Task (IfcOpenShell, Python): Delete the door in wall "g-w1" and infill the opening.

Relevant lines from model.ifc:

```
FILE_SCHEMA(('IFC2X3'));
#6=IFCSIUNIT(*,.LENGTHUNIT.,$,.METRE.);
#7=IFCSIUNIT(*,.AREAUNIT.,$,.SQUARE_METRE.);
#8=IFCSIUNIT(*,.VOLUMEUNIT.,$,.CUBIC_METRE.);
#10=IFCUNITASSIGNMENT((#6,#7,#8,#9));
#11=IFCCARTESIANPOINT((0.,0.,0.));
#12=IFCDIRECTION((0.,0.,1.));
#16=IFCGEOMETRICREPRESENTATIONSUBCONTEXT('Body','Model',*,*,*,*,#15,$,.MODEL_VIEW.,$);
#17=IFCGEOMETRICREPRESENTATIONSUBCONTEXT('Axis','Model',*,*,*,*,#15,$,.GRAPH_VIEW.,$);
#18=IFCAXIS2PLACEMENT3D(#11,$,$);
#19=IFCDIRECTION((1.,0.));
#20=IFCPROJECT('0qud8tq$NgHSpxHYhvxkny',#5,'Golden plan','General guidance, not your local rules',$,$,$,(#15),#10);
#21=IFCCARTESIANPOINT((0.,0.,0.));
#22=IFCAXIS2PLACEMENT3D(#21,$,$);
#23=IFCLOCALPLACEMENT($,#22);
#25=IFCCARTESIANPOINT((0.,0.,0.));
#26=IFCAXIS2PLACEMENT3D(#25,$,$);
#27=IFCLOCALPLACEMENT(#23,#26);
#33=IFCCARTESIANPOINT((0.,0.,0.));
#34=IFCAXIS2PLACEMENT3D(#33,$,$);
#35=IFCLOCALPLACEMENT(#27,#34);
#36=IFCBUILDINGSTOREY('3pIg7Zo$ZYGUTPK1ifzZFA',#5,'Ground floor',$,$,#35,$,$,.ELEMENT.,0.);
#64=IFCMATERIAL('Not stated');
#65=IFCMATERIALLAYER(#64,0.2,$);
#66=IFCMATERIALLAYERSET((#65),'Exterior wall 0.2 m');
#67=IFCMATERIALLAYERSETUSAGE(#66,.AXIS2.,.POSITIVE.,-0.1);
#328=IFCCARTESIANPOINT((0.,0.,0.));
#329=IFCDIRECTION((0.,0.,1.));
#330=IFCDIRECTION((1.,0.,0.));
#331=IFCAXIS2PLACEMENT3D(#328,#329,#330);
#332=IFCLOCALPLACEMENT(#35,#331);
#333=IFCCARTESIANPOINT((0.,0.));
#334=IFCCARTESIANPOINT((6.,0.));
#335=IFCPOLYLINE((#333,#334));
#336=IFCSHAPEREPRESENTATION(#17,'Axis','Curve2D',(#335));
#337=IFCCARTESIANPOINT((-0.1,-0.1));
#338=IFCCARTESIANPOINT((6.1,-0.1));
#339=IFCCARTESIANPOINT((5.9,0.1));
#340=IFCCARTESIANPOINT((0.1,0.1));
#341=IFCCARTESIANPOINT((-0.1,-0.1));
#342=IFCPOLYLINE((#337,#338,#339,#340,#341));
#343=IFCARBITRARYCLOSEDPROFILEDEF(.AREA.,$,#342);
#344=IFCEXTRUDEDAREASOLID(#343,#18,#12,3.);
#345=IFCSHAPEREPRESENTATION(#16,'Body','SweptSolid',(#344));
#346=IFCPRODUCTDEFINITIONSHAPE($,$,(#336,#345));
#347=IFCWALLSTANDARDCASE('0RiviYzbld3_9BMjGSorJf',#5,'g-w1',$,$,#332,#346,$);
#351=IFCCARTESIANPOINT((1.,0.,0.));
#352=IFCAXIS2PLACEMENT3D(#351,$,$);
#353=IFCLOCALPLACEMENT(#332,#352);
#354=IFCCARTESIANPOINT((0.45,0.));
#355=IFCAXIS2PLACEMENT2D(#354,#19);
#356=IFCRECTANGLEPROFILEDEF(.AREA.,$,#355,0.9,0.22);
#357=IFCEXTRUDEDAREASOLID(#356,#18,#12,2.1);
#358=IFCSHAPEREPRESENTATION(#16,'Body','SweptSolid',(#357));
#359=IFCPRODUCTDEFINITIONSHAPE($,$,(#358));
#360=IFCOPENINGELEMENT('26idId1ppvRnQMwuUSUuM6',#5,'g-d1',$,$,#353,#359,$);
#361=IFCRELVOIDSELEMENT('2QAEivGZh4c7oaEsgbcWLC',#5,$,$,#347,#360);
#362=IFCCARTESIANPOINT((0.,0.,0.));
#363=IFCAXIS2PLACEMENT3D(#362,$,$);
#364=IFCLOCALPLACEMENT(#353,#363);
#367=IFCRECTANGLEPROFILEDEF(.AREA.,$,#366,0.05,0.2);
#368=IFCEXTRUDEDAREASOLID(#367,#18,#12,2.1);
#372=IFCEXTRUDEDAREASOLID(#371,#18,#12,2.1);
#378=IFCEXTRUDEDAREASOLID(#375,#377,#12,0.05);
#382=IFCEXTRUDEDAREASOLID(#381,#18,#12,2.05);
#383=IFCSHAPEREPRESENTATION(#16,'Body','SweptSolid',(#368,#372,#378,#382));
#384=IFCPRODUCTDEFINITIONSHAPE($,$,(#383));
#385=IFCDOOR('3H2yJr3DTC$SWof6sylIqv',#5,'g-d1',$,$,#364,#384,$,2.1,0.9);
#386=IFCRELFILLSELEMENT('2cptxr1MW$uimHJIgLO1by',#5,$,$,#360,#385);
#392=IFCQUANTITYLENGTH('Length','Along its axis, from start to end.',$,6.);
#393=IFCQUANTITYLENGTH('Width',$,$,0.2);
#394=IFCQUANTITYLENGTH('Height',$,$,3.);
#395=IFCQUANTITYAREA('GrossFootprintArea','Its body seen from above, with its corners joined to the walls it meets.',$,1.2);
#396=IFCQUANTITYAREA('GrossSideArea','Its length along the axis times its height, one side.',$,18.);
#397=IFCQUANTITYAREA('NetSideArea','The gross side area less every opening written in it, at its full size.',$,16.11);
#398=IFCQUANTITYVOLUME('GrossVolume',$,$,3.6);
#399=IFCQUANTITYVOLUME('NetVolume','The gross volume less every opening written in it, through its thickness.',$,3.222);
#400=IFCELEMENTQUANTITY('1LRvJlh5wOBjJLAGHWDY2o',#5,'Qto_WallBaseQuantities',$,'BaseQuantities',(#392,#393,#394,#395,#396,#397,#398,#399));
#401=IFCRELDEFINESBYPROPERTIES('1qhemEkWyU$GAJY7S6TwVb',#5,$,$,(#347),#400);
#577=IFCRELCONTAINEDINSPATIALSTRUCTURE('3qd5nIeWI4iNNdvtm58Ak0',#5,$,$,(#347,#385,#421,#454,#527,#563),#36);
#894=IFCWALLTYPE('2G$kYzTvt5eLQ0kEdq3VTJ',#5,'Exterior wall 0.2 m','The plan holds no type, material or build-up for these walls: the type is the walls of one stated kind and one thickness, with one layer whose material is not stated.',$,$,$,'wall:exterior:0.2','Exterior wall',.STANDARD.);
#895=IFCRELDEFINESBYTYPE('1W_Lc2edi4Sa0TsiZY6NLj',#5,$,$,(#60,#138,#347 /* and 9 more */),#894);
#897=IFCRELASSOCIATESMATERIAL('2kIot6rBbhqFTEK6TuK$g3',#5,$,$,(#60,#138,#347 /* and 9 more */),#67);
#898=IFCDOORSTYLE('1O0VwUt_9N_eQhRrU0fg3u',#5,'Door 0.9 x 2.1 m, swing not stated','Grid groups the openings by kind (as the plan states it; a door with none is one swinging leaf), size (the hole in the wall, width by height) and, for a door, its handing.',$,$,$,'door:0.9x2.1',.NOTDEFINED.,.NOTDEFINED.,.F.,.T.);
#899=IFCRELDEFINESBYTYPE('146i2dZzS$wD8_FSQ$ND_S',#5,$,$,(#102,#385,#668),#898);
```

```python
import ifcopenshell
import ifcopenshell.api.feature
import ifcopenshell.api.pset
import ifcopenshell.api.root
import ifcopenshell.geom
import ifcopenshell.util.element
import ifcopenshell.util.shape
import ifcopenshell.util.unit

model = ifcopenshell.open("model.ifc")
area_scale = ifcopenshell.util.unit.calculate_unit_scale(model, "AREAUNIT")
volume_scale = ifcopenshell.util.unit.calculate_unit_scale(model, "VOLUMEUNIT")
settings = ifcopenshell.geom.settings()


def volume(element):
    """Net volume in cubic metres, openings subtracted."""
    shape = ifcopenshell.geom.create_shape(settings, element)
    return ifcopenshell.util.shape.get_volume(shape.geometry)


door = model.by_id(385)
opening = door.FillsVoids[0].RelatingOpeningElement
wall = opening.VoidsElements[0].RelatingBuildingElement
before = volume(wall)

ifcopenshell.api.root.remove_product(model, product=door)
ifcopenshell.api.feature.remove_feature(model, feature=opening)

after = volume(wall)
thickness = 0.2  # wall thickness in metres

# Update the wall's stored quantities.
qto = model.by_id(ifcopenshell.util.element.get_pset(wall, "Qto_WallBaseQuantities", should_inherit=False)["id"])
ifcopenshell.api.pset.edit_qto(model, qto=qto, properties={
    "NetSideArea": after / thickness / area_scale,
    "NetVolume": after / volume_scale,
})

print(f"wall volume {before:.3f} -> {after:.3f} m3")

model.write("model_rev.ifc")
```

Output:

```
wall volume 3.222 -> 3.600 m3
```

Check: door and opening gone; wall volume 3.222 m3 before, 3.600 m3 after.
